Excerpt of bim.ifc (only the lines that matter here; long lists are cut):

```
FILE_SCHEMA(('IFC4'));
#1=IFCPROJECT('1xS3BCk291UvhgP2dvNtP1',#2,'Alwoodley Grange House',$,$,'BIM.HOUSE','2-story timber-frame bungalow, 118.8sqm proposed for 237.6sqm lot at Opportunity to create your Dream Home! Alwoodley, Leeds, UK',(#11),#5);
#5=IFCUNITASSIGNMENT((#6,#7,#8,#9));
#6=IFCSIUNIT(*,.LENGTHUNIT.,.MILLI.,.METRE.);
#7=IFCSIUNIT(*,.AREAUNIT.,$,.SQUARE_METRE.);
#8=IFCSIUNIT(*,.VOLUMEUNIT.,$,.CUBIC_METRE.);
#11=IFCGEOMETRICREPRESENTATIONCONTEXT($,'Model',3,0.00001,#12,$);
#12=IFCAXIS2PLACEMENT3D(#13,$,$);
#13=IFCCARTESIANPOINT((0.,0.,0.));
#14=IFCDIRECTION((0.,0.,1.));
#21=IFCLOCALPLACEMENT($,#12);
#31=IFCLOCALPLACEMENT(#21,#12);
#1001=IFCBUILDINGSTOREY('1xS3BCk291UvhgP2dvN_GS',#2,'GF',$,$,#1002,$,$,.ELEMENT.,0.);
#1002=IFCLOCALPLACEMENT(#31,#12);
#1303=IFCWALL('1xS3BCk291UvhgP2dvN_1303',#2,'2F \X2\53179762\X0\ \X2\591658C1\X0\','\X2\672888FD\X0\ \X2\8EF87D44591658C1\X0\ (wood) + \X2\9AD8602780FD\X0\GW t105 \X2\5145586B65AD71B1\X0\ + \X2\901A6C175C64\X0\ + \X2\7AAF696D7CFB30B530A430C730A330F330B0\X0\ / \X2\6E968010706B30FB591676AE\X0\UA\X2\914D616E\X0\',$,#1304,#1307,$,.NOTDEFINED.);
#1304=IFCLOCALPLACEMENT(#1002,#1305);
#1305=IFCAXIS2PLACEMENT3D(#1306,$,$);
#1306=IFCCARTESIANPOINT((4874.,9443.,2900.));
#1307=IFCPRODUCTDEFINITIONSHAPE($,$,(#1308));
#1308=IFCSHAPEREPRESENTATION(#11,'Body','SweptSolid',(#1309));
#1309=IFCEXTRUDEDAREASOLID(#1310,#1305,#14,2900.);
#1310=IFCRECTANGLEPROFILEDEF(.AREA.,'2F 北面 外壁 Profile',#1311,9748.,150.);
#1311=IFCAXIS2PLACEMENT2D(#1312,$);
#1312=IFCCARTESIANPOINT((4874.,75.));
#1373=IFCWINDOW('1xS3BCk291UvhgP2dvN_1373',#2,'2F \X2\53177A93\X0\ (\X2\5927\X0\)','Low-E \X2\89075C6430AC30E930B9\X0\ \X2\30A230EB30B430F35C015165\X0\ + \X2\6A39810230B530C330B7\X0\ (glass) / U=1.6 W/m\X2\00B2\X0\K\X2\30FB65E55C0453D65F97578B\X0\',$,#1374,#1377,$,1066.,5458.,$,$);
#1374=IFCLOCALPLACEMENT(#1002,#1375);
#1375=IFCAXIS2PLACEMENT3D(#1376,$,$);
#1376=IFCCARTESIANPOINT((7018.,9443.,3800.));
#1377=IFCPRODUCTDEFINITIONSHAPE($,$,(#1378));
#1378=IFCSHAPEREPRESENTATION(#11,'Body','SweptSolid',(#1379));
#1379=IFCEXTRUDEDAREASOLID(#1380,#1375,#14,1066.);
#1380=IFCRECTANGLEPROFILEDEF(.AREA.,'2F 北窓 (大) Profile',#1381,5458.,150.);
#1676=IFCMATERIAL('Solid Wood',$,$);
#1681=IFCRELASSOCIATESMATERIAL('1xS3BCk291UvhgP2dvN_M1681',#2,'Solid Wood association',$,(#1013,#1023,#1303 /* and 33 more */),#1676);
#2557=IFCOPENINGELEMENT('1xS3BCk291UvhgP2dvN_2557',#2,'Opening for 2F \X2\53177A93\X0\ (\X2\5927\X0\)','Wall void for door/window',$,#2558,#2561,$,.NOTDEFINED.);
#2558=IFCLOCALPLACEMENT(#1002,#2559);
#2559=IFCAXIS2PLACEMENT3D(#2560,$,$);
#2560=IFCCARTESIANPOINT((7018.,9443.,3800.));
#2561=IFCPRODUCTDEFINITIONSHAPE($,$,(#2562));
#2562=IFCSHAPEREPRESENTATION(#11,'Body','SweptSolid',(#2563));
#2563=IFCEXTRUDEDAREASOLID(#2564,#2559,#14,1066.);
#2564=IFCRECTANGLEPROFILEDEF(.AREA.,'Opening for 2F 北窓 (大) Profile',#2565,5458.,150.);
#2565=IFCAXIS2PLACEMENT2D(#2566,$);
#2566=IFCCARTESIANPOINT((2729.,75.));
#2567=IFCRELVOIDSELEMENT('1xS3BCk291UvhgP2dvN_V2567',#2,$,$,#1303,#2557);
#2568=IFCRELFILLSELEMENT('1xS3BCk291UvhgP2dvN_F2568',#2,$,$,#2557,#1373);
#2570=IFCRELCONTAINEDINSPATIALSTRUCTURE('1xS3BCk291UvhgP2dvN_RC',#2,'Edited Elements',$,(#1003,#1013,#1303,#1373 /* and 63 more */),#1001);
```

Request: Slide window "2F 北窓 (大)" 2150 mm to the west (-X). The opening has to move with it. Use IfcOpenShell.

```python
import ifcopenshell
import ifcopenshell.api.geometry
import ifcopenshell.util.placement
import ifcopenshell.util.unit

model = ifcopenshell.open("bim.ifc")
unit_scale = ifcopenshell.util.unit.calculate_unit_scale(model)

window = model.by_guid("1xS3BCk291UvhgP2dvN_1373")
opening = window.FillsVoids[0].RelatingOpeningElement
wall = opening.VoidsElements[0].RelatingBuildingElement

wall_matrix = ifcopenshell.util.placement.get_local_placement(wall.ObjectPlacement)
shift = wall_matrix[:3, 0] * -2.15 / unit_scale
before = ifcopenshell.util.placement.get_local_placement(window.ObjectPlacement)[:3, 3].copy()

# The window is not placed relative to its opening, so move both.
for product in (opening, window):
    matrix = ifcopenshell.util.placement.get_local_placement(product.ObjectPlacement)
    matrix[:3, 3] += shift
    ifcopenshell.api.geometry.edit_object_placement(model, product=product, matrix=matrix, is_si=False)

after = ifcopenshell.util.placement.get_local_placement(window.ObjectPlacement)[:3, 3]
print("window moved by", (after - before).round(3) + 0.0)

model.write("bim-out.ifc")
```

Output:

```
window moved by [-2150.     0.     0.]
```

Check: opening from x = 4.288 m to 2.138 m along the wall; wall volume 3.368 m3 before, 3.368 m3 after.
